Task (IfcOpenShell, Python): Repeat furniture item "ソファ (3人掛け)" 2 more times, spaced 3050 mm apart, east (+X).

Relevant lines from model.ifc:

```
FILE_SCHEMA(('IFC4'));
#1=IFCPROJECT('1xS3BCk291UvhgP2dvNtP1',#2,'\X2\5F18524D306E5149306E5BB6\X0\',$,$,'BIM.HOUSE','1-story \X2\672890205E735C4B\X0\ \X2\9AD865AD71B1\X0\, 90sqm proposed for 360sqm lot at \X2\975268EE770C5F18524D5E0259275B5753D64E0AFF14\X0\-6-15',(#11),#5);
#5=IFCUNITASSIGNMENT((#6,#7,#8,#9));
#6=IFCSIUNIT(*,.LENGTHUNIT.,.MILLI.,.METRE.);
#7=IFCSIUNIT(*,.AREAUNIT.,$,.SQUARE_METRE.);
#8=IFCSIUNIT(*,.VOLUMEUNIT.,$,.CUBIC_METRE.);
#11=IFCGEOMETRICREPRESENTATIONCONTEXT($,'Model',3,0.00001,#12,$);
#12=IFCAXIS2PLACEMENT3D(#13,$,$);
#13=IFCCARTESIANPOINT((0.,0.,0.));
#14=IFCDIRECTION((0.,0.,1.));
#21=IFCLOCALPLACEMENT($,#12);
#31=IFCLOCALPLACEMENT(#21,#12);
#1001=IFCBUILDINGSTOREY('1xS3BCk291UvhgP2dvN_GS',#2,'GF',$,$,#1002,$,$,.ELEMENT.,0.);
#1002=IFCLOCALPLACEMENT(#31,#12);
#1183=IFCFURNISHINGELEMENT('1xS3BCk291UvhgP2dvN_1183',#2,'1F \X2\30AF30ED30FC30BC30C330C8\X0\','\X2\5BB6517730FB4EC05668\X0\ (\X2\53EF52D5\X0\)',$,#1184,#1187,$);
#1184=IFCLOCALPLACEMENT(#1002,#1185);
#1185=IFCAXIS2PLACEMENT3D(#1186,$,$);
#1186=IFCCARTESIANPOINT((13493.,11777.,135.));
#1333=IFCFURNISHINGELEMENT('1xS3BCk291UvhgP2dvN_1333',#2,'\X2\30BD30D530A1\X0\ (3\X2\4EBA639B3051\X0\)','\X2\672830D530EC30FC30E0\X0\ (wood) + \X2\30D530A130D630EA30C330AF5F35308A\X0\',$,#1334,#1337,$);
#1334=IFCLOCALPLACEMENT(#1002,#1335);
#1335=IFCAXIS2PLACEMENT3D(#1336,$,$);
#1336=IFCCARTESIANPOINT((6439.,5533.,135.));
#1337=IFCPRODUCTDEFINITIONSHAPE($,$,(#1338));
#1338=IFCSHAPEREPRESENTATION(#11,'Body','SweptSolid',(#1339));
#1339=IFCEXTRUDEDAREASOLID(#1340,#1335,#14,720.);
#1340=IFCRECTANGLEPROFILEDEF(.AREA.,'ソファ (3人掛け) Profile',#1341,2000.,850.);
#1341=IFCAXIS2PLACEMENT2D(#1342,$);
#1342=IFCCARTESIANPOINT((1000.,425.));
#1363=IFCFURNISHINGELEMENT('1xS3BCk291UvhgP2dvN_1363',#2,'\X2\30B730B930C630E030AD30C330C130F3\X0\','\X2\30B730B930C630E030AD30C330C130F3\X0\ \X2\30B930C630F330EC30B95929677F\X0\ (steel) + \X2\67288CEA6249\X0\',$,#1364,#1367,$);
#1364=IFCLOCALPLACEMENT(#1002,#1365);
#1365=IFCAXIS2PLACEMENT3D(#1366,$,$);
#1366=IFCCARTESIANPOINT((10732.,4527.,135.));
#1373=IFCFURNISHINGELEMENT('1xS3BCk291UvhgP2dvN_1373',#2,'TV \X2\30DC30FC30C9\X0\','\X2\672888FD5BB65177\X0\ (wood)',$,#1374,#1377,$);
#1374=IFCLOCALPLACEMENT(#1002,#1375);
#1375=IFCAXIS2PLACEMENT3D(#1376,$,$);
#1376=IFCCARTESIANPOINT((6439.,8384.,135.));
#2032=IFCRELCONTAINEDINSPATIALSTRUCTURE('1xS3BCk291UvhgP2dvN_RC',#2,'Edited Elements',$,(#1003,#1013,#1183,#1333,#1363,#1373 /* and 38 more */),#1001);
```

```python
import numpy as np
import ifcopenshell
import ifcopenshell.api.geometry
import ifcopenshell.api.root
import ifcopenshell.util.element
import ifcopenshell.util.placement

model = ifcopenshell.open("model.ifc")


def reuse_history(source, copy):
    """copy_class also copies each property set's owner history, people and application; keep the originals."""
    for rel in copy.IsDefinedBy:
        if rel.is_a("IfcRelDefinesByProperties") and (history := rel.RelatingPropertyDefinition.OwnerHistory):
            rel.RelatingPropertyDefinition.OwnerHistory = source.OwnerHistory
            ifcopenshell.util.element.remove_deep2(model, history)


source = model.by_guid("1xS3BCk291UvhgP2dvN_1333")
base = ifcopenshell.util.placement.get_local_placement(source.ObjectPlacement)
step = np.array([1.0, 0.0, 0.0]) * 3050.0

for i in range(1, 3):
    copy = ifcopenshell.api.root.copy_class(model, product=source)
    copy.Representation = ifcopenshell.util.element.copy_deep(
        model, source.Representation, exclude=["IfcGeometricRepresentationContext", "IfcRepresentationMap"]
    )
    reuse_history(source, copy)
    matrix = base.copy()
    matrix[:3, 3] += i * step
    print("added at", matrix[:3, 3].round(3) + 0.0)
    ifcopenshell.api.geometry.edit_object_placement(model, product=copy, matrix=matrix, is_si=False)

model.write("model_updated.ifc")
```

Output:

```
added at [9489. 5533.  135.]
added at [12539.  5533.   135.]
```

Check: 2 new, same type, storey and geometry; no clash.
